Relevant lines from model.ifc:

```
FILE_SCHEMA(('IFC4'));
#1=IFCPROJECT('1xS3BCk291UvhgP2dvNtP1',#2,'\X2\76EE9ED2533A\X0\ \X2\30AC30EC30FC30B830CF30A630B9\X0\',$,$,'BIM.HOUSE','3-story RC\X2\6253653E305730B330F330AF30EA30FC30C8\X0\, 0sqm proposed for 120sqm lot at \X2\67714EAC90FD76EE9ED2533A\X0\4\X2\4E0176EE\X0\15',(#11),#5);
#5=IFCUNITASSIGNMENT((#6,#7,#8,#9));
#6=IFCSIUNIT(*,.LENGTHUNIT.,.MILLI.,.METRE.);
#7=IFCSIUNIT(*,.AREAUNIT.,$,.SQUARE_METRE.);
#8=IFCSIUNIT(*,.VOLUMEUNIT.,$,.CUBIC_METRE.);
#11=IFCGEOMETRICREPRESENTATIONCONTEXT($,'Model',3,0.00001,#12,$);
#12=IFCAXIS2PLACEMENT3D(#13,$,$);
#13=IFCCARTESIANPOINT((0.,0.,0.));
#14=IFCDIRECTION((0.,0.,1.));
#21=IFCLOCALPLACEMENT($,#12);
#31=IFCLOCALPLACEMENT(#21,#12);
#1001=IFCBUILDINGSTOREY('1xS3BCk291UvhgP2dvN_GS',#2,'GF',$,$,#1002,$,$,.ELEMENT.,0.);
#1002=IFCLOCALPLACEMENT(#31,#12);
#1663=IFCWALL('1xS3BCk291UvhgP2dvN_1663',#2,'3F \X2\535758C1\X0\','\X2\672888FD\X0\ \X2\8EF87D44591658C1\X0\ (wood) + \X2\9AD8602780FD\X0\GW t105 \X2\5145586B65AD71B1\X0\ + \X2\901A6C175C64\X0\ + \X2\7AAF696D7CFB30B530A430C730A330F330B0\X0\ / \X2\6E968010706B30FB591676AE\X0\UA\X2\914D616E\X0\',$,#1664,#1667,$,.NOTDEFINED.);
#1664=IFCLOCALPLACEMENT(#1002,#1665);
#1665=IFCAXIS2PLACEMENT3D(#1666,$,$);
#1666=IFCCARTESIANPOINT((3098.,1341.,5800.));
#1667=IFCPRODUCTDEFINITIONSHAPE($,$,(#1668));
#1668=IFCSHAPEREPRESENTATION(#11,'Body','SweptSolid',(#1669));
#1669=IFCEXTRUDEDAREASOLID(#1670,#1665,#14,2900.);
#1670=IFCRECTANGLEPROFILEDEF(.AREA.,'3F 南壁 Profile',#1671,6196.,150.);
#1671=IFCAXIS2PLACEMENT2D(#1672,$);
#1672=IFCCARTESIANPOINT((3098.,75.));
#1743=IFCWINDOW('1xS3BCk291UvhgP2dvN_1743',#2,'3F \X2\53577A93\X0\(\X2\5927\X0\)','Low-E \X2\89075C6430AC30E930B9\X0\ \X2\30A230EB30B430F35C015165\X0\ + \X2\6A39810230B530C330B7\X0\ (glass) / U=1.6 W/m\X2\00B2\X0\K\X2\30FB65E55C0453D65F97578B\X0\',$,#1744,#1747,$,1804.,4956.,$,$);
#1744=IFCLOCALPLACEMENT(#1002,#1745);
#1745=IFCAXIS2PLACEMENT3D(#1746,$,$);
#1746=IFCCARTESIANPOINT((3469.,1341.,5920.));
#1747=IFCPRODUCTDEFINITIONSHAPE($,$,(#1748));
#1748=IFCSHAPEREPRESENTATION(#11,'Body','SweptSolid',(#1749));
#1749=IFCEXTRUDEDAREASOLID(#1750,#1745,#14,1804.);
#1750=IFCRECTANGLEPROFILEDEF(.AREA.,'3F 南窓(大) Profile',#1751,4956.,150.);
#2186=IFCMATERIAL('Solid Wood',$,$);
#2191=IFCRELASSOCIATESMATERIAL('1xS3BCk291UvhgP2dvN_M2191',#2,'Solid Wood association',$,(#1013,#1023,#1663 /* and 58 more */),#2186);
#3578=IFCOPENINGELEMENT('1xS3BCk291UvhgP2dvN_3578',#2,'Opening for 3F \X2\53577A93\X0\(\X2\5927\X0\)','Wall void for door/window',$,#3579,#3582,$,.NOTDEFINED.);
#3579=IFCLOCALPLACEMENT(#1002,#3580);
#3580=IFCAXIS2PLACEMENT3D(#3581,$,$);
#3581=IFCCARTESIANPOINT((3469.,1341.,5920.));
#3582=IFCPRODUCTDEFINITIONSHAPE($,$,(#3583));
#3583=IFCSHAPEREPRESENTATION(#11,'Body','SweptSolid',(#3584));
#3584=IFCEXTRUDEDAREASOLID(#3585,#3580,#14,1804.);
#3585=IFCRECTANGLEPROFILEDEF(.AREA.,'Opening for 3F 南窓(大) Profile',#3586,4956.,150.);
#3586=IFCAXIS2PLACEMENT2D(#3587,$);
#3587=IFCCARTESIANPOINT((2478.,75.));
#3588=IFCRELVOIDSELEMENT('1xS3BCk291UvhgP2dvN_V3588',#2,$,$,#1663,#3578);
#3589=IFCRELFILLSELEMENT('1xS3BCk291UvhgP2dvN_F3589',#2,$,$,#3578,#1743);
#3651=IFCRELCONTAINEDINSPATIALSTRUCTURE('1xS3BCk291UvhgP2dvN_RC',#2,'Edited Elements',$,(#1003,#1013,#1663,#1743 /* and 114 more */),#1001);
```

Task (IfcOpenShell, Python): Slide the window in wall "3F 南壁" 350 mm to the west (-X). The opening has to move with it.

```python
import ifcopenshell
import ifcopenshell.api.geometry
import ifcopenshell.util.placement
import ifcopenshell.util.unit

model = ifcopenshell.open("model.ifc")
unit_scale = ifcopenshell.util.unit.calculate_unit_scale(model)

window = model.by_guid("1xS3BCk291UvhgP2dvN_1743")
opening = window.FillsVoids[0].RelatingOpeningElement
wall = opening.VoidsElements[0].RelatingBuildingElement

wall_matrix = ifcopenshell.util.placement.get_local_placement(wall.ObjectPlacement)
shift = wall_matrix[:3, 0] * -0.35 / unit_scale
before = ifcopenshell.util.placement.get_local_placement(window.ObjectPlacement)[:3, 3].copy()

# The window is not placed relative to its opening, so move both.
for product in (opening, window):
    matrix = ifcopenshell.util.placement.get_local_placement(product.ObjectPlacement)
    matrix[:3, 3] += shift
    ifcopenshell.api.geometry.edit_object_placement(model, product=product, matrix=matrix, is_si=False)

after = ifcopenshell.util.placement.get_local_placement(window.ObjectPlacement)[:3, 3]
print("window moved by", (after - before).round(3) + 0.0)

model.write("model_rev.ifc")
```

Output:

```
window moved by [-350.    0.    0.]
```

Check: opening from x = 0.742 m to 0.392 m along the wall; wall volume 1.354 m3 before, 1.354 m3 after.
